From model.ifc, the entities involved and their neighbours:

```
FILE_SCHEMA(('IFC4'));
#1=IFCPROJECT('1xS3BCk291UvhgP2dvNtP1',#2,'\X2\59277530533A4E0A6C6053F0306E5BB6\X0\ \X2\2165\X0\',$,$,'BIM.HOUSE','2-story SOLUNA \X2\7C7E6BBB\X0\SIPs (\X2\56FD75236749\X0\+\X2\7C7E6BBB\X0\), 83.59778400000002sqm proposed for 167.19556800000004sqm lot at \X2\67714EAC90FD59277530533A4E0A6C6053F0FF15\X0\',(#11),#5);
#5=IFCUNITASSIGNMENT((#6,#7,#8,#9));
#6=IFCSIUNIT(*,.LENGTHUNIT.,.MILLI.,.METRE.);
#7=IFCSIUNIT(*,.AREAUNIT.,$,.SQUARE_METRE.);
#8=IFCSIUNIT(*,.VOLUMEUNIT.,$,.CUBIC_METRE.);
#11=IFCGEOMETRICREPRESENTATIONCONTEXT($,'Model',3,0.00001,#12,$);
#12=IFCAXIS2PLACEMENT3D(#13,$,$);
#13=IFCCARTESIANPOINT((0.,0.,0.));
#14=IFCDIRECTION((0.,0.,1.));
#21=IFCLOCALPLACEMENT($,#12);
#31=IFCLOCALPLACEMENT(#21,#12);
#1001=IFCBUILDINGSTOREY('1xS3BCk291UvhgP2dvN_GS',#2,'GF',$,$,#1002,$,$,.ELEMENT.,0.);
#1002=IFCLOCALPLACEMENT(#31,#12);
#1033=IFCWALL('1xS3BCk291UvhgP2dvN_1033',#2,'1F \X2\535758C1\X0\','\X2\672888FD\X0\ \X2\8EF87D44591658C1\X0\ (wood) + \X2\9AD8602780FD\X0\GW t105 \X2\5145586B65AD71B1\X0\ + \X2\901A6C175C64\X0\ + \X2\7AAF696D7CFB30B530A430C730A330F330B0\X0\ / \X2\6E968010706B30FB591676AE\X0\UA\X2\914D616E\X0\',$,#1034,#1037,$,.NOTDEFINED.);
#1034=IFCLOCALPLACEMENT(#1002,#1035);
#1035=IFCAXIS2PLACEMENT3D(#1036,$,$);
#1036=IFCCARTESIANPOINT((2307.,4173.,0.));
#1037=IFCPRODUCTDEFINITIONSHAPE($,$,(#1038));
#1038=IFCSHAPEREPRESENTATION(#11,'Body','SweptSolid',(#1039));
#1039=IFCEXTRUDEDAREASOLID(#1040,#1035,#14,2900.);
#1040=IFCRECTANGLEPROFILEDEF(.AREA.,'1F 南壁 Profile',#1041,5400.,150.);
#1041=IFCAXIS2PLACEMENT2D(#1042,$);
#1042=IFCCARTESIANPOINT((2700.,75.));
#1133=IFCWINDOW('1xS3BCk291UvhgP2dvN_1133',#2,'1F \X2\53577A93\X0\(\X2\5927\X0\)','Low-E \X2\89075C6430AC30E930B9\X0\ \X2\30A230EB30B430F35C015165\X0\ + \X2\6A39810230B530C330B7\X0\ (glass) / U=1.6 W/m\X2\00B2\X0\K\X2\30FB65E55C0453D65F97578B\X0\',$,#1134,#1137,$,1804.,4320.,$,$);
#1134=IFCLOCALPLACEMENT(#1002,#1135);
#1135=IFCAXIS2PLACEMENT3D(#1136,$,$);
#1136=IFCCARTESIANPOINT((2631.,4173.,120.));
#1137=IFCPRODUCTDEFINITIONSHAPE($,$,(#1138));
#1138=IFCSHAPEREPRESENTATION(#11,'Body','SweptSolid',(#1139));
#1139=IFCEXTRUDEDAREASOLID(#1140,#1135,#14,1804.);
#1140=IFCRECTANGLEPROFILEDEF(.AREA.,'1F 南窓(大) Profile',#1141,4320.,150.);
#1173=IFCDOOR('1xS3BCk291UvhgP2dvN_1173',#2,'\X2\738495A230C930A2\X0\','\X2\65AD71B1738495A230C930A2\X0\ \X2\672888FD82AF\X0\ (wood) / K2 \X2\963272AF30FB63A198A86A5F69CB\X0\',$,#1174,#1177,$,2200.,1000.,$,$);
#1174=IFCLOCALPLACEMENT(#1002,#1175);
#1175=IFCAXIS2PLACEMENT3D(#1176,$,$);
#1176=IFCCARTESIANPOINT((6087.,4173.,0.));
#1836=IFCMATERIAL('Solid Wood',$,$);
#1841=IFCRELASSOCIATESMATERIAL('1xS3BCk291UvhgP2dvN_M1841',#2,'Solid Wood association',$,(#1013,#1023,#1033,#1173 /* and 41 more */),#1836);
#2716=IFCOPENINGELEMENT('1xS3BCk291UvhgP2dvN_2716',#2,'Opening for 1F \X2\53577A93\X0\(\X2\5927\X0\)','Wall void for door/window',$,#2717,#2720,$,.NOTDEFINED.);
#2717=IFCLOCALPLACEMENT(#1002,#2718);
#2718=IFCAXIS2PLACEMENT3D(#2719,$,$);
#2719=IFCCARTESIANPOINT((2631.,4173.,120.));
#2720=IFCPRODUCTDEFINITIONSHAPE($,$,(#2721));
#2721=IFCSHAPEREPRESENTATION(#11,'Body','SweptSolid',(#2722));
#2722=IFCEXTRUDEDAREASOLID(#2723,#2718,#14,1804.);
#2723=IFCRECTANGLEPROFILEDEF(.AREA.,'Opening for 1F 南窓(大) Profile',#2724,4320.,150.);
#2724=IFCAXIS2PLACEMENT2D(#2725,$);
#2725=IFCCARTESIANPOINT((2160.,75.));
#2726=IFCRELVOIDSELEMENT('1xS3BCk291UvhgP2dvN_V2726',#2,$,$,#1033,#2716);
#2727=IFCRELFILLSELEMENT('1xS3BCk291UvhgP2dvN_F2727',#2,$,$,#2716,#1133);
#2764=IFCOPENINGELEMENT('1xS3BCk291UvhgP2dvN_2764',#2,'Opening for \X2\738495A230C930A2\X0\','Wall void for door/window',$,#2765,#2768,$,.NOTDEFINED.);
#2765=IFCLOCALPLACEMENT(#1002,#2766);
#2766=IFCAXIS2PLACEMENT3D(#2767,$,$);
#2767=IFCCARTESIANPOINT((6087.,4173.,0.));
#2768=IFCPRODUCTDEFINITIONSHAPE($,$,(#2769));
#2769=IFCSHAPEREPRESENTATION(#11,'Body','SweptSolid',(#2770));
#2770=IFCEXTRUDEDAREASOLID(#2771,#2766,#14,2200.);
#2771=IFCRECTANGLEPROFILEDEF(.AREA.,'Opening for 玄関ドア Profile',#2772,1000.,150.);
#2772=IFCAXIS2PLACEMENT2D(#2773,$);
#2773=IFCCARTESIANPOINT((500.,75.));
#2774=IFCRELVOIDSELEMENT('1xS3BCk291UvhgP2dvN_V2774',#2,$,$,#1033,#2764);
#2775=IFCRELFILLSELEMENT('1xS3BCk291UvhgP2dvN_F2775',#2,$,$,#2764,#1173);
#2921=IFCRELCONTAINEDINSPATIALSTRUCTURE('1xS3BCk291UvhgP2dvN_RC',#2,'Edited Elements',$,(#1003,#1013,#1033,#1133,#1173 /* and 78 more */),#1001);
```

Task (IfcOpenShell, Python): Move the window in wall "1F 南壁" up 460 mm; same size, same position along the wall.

```python
import numpy as np
import ifcopenshell
import ifcopenshell.api.geometry
import ifcopenshell.util.placement
import ifcopenshell.util.unit

model = ifcopenshell.open("model.ifc")
unit_scale = ifcopenshell.util.unit.calculate_unit_scale(model)

window = model.by_id(1133)
opening = window.FillsVoids[0].RelatingOpeningElement
dz = 0.46 / unit_scale

shift = np.array([0.0, 0.0, dz])
# The window is not placed relative to its opening, so move both.
for product in (opening, window):
    matrix = ifcopenshell.util.placement.get_local_placement(product.ObjectPlacement)
    matrix[:3, 3] += shift
    ifcopenshell.api.geometry.edit_object_placement(model, product=product, matrix=matrix, is_si=False)

print(f"moved by {dz * unit_scale:+.3f} m")

model.write("model_edited.ifc")
```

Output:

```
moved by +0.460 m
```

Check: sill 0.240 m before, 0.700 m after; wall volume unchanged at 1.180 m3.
